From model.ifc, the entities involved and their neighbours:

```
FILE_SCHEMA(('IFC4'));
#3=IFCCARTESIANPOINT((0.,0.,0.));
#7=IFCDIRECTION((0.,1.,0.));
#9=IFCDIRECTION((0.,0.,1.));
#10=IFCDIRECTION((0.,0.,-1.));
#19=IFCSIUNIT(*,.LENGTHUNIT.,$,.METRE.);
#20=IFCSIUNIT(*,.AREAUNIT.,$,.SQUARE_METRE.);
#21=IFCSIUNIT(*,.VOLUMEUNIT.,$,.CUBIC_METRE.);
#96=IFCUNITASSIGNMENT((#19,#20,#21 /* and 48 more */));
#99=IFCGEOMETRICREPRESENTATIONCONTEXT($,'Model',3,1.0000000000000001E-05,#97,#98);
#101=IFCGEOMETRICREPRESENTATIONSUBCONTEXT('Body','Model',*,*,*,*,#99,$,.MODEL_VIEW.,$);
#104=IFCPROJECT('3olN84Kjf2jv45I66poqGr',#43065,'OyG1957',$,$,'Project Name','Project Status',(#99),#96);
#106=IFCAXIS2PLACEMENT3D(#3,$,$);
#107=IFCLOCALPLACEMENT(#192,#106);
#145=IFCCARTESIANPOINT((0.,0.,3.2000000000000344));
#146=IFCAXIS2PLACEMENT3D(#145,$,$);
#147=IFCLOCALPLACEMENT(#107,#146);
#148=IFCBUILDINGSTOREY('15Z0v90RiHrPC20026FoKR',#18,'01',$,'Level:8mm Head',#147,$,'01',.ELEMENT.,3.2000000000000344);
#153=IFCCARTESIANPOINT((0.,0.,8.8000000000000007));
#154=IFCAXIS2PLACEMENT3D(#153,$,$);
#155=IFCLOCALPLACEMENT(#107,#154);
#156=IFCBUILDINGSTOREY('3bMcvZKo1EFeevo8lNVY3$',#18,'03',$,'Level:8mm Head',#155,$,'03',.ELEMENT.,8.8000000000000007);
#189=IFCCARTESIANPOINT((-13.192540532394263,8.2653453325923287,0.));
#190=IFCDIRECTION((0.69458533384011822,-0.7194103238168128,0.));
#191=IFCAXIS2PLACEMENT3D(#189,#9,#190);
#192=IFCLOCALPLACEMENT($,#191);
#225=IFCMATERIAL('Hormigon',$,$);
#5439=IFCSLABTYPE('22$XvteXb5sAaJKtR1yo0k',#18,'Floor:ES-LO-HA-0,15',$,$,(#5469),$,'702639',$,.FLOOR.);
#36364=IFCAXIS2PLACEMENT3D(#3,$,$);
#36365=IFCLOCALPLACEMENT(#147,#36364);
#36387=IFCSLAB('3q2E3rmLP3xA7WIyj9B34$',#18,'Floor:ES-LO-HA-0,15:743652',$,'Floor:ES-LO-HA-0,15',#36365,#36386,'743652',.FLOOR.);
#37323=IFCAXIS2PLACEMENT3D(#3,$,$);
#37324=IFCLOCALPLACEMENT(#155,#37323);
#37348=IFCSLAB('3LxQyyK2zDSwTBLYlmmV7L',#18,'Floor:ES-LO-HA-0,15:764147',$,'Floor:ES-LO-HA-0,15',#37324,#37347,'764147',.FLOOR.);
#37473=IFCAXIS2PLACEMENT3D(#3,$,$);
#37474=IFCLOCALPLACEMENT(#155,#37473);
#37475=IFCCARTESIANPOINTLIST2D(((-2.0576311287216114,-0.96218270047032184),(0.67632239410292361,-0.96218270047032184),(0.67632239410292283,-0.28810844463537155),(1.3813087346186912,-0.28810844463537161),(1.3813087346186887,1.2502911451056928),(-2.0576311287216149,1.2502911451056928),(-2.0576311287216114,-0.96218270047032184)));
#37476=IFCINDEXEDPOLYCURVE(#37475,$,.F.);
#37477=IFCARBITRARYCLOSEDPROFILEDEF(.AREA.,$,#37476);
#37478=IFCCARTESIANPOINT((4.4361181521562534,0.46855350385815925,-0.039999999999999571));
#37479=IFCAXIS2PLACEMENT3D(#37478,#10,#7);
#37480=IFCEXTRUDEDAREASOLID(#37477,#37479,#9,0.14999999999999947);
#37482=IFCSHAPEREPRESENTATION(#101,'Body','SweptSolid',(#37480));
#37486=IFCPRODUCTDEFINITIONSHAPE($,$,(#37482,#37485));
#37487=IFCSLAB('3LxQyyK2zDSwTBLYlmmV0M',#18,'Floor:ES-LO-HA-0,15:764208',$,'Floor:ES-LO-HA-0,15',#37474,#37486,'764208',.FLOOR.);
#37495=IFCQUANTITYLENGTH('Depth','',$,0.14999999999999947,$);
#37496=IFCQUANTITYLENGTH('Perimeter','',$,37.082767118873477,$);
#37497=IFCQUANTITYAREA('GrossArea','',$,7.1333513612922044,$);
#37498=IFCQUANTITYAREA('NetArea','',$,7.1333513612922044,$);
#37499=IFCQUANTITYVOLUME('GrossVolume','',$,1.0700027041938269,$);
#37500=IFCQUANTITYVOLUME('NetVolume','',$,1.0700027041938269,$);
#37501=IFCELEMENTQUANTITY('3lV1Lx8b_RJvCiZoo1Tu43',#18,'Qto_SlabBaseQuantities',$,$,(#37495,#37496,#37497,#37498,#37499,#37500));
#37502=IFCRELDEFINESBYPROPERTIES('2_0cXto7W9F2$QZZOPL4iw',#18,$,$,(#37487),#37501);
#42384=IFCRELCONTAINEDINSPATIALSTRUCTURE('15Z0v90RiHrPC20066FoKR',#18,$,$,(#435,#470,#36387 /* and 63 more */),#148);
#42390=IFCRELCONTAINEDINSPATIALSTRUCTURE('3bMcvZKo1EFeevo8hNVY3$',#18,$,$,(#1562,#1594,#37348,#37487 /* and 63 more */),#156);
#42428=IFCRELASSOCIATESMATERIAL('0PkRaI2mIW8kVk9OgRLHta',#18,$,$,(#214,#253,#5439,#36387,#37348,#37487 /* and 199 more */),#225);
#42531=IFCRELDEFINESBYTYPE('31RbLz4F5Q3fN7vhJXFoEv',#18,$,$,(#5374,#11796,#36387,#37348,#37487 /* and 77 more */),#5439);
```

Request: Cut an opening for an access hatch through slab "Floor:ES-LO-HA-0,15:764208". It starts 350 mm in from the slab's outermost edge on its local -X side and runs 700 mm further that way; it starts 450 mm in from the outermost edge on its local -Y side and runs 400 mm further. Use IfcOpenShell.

```python
import numpy as np
import ifcopenshell
import ifcopenshell.api.feature
import ifcopenshell.api.geometry
import ifcopenshell.api.pset
import ifcopenshell.api.root
import ifcopenshell.geom
import ifcopenshell.util.element
import ifcopenshell.util.placement
import ifcopenshell.util.representation
import ifcopenshell.util.shape
import ifcopenshell.util.unit

model = ifcopenshell.open("model.ifc")
unit_scale = ifcopenshell.util.unit.calculate_unit_scale(model)
area_scale = ifcopenshell.util.unit.calculate_unit_scale(model, "AREAUNIT")
volume_scale = ifcopenshell.util.unit.calculate_unit_scale(model, "VOLUMEUNIT")
settings = ifcopenshell.geom.settings()


def volume(element):
    """Net volume in cubic metres, openings subtracted."""
    shape = ifcopenshell.geom.create_shape(settings, element)
    return ifcopenshell.util.shape.get_volume(shape.geometry)


slab = model.by_guid("3LxQyyK2zDSwTBLYlmmV0M")
before = volume(slab)

# Extent in the slab's own axes, in metres. The edges named are its -X and -Y sides.
slab_shape = ifcopenshell.geom.create_shape(settings, slab)
vertices = ifcopenshell.util.shape.get_vertices(slab_shape.geometry)
x_min, y_min, bottom = vertices.min(axis=0)
top = vertices[:, 2].max()

opening = ifcopenshell.api.root.create_entity(model, ifc_class="IfcOpeningElement", name="Access hatch opening", predefined_type="OPENING")
context = ifcopenshell.util.representation.get_context(model, "Model", "Body", "MODEL_VIEW")
width, depth = 0.7, 0.4
outline = [(0.0, 0.0), (width, 0.0), (width, depth), (0.0, depth), (0.0, 0.0)]
# Overshoot both faces by 50 mm so the cut is clean.
shape = ifcopenshell.api.geometry.add_slab_representation(
    model, context=context, depth=top - bottom + 0.1, polyline=outline
)
ifcopenshell.api.geometry.assign_representation(model, product=opening, representation=shape)

matrix = ifcopenshell.util.placement.get_local_placement(slab.ObjectPlacement)
matrix[:, 3] = matrix @ np.append(np.array([x_min + 0.35, y_min + 0.45, bottom - 0.05]) / unit_scale, 1.0)
ifcopenshell.api.geometry.edit_object_placement(model, product=opening, matrix=matrix, is_si=False)
ifcopenshell.api.feature.add_feature(model, feature=opening, element=slab)

after = volume(slab)

# Update the slab's stored quantities.
qto = model.by_id(ifcopenshell.util.element.get_pset(slab, "Qto_SlabBaseQuantities", should_inherit=False)["id"])
ifcopenshell.api.pset.edit_qto(model, qto=qto, properties={
    "NetArea": after / (top - bottom) / area_scale,
    "NetVolume": after / volume_scale,
})

print(f"slab volume {before:.3f} -> {after:.3f} m3")

model.write("model_v2.ifc")
```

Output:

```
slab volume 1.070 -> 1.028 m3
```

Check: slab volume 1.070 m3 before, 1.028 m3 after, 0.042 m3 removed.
